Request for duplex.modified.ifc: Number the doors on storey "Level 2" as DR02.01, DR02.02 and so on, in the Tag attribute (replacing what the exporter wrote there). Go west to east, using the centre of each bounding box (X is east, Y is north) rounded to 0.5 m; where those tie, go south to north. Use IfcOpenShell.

First a look at what the model holds.

```python
import ifcopenshell
import ifcopenshell.util.element
import ifcopenshell.util.placement

model = ifcopenshell.open("duplex.modified.ifc")
print(model.schema)
storey = next(s for s in model.by_type("IfcBuildingStorey") if s.Name == "Level 2")
doors = [e for e in ifcopenshell.util.element.get_decomposition(storey) if e.is_a("IfcDoor")]
for e in sorted(doors, key=lambda e: e.id()):
    origin = ifcopenshell.util.placement.get_local_placement(e.ObjectPlacement)[:3, 3]
    print(e.id(), e.Tag, e.Name, origin.round(2) + 0.0, sep=" | ")
```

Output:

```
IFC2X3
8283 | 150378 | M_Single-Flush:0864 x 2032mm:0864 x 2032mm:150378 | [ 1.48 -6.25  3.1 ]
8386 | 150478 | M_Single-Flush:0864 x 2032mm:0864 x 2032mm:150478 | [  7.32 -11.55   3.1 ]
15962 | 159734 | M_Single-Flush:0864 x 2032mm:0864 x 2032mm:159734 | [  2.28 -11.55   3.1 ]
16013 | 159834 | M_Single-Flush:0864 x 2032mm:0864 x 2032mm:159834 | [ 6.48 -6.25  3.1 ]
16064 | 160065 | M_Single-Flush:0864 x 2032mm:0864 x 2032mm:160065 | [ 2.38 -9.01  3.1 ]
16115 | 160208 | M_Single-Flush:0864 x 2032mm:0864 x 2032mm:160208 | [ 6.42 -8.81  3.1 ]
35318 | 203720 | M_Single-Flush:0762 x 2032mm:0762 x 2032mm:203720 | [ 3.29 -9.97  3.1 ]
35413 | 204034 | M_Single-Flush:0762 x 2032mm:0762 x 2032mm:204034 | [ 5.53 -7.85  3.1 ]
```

```python
import ifcopenshell
import ifcopenshell.geom
import ifcopenshell.util.element
import ifcopenshell.util.shape

model = ifcopenshell.open("duplex.modified.ifc")
settings = ifcopenshell.geom.settings()
settings.set("use-world-coords", True)


def centre(element):
    shape = ifcopenshell.geom.create_shape(settings, element)
    return ifcopenshell.util.shape.get_bbox_centroid(shape.geometry)


storey = next(s for s in model.by_type("IfcBuildingStorey") if s.Name == "Level 2")
doors = [e for e in ifcopenshell.util.element.get_decomposition(storey) if e.is_a("IfcDoor")]

# Insertion points can sit at a corner or the storey origin, so sort by the geometry (in metres).
centres = {e: centre(e) for e in doors}
doors.sort(key=lambda e: (round(centres[e][0] / 0.5), centres[e][1]))

for i, e in enumerate(doors, start=1):
    number = f"DR02.{i:02d}"
    e.Tag = number
    print(e.id(), number)

model.write("duplex.modified_updated.ifc")
```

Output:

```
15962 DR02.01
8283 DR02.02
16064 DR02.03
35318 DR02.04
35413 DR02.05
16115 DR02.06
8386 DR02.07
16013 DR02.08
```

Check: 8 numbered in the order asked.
